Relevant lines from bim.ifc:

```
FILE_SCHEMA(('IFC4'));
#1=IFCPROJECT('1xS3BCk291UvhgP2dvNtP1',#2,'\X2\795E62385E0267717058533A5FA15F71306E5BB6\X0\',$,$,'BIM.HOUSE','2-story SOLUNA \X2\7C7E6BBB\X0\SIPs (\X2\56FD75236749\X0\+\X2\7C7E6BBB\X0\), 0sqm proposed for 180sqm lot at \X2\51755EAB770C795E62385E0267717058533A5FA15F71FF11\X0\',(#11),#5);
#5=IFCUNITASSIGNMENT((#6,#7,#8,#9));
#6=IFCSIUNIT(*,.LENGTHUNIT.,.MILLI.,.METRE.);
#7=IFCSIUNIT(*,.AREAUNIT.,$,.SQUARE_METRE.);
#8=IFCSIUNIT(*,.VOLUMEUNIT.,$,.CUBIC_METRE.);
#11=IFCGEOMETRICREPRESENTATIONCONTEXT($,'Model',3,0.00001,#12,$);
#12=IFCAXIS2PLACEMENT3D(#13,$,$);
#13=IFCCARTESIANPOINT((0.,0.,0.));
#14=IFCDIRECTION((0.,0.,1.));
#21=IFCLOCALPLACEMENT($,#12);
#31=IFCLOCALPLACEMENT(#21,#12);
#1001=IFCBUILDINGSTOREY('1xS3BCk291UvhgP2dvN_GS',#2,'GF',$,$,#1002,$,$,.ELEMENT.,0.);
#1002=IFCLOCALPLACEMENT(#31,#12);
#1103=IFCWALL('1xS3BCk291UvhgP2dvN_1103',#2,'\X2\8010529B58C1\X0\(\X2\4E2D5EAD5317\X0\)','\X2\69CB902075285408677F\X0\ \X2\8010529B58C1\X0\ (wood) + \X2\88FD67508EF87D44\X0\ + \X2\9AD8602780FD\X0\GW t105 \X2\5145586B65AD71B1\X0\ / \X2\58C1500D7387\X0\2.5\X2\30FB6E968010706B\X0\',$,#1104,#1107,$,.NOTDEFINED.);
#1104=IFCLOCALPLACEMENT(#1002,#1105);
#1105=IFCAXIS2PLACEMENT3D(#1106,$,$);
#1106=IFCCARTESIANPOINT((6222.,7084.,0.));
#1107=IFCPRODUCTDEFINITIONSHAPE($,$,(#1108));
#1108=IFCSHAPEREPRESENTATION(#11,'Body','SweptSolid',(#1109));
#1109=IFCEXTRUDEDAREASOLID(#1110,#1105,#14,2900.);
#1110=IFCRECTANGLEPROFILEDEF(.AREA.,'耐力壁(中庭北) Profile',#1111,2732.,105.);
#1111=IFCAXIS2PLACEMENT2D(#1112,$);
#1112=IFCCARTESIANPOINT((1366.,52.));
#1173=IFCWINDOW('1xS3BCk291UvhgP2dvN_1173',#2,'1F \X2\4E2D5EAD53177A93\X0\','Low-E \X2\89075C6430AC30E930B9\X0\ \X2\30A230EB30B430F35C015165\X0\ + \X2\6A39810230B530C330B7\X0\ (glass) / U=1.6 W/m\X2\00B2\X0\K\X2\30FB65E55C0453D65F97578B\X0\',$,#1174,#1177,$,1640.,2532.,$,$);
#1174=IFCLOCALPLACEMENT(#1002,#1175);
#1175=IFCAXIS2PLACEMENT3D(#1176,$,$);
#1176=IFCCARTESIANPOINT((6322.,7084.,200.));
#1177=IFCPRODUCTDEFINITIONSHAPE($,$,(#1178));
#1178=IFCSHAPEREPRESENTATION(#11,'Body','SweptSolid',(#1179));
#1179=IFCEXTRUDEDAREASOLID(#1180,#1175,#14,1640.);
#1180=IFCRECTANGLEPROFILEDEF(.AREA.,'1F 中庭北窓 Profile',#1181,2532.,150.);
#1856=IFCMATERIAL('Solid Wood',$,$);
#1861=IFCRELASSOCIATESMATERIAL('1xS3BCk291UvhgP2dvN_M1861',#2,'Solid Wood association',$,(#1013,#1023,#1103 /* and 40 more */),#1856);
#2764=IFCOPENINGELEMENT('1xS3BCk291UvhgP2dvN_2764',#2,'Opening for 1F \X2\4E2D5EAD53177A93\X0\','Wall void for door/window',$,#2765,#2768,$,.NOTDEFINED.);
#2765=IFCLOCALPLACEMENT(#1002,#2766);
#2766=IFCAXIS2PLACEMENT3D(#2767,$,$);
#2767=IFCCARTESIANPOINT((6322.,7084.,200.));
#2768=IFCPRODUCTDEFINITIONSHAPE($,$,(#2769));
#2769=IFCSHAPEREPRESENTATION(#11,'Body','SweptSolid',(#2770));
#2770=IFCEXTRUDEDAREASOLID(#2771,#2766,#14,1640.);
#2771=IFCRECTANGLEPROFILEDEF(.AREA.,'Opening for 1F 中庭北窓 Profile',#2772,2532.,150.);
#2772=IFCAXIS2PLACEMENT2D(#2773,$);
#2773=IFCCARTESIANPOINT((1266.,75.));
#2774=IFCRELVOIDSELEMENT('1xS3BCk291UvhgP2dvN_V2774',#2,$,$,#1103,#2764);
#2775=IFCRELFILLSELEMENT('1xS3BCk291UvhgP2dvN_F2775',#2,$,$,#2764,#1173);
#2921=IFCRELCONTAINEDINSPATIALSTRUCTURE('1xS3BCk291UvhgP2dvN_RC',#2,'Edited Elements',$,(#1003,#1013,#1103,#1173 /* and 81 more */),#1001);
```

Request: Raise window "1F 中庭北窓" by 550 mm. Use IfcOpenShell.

```python
import numpy as np
import ifcopenshell
import ifcopenshell.api.geometry
import ifcopenshell.util.placement
import ifcopenshell.util.unit

model = ifcopenshell.open("bim.ifc")
unit_scale = ifcopenshell.util.unit.calculate_unit_scale(model)

window = model.by_guid("1xS3BCk291UvhgP2dvN_1173")
opening = window.FillsVoids[0].RelatingOpeningElement
dz = 0.55 / unit_scale

shift = np.array([0.0, 0.0, dz])
# The window is not placed relative to its opening, so move both.
for product in (opening, window):
    matrix = ifcopenshell.util.placement.get_local_placement(product.ObjectPlacement)
    matrix[:3, 3] += shift
    ifcopenshell.api.geometry.edit_object_placement(model, product=product, matrix=matrix, is_si=False)

print(f"moved by {dz * unit_scale:+.3f} m")

model.write("bim_rev.ifc")
```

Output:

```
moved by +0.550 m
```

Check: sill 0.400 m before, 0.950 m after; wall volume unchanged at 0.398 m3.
